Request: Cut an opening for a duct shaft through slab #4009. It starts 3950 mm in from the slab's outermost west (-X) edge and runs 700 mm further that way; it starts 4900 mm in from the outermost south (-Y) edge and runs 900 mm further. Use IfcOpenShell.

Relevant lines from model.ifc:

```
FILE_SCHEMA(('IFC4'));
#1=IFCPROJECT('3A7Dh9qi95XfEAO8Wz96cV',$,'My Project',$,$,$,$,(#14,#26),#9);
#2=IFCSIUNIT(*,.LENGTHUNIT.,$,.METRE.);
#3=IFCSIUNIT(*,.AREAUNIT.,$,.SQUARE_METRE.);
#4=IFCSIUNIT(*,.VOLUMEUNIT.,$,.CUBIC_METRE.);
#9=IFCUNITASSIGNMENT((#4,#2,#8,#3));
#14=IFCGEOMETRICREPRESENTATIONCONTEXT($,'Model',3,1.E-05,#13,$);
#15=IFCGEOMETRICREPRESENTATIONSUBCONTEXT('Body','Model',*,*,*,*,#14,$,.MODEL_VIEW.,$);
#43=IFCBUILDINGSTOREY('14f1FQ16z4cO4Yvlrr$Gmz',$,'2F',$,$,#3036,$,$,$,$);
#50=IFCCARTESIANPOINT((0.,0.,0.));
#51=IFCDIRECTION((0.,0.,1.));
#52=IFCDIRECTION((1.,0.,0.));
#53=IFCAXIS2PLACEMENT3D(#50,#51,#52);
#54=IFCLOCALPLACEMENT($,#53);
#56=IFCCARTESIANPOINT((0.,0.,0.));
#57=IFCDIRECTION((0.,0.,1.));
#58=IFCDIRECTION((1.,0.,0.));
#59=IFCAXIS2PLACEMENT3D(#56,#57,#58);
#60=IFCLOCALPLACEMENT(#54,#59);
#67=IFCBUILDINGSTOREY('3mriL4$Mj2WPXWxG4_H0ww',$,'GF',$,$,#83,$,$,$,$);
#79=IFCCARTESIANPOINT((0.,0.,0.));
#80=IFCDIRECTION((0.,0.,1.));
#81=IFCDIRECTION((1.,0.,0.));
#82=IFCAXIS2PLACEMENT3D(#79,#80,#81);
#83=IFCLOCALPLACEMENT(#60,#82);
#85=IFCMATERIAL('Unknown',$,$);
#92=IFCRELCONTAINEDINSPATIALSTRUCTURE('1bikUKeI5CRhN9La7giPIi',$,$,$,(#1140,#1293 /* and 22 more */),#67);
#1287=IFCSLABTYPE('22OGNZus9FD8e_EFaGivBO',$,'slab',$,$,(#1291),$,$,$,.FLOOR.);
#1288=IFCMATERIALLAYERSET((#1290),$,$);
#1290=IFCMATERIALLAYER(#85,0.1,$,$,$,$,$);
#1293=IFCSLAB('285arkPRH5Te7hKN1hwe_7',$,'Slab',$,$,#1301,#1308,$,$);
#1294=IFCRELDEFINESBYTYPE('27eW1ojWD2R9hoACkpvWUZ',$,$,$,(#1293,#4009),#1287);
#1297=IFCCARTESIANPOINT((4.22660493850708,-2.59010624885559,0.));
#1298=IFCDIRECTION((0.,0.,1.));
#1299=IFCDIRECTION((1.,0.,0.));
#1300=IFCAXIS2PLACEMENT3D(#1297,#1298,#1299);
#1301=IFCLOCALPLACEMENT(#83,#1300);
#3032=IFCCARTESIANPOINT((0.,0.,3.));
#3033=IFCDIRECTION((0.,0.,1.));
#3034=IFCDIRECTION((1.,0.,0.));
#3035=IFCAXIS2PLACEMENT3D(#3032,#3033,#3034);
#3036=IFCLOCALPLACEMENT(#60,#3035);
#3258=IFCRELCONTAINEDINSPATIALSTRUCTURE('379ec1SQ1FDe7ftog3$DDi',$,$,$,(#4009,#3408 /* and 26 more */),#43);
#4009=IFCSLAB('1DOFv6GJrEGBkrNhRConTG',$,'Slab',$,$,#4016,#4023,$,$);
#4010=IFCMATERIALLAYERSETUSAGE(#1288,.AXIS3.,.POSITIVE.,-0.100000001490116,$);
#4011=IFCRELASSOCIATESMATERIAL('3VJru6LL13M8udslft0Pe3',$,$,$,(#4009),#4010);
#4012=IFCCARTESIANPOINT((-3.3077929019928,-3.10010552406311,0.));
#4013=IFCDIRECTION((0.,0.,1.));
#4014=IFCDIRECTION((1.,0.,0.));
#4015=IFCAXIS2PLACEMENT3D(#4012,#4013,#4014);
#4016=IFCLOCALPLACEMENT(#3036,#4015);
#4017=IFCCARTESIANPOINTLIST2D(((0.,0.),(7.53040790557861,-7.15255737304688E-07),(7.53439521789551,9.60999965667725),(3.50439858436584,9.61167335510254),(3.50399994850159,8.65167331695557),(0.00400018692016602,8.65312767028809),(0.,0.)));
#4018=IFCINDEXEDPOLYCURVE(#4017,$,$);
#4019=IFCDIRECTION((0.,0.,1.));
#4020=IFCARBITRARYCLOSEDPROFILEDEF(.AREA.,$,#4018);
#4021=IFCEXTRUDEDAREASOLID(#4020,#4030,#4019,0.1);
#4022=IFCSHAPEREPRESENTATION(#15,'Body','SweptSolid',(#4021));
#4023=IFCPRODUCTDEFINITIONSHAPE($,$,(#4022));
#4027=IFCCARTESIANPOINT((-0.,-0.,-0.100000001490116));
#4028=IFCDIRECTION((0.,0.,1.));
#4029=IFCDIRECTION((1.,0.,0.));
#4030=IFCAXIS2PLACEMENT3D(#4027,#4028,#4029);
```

```python
import numpy as np
import ifcopenshell
import ifcopenshell.api.feature
import ifcopenshell.api.geometry
import ifcopenshell.api.root
import ifcopenshell.geom
import ifcopenshell.util.placement
import ifcopenshell.util.representation
import ifcopenshell.util.shape
import ifcopenshell.util.unit

model = ifcopenshell.open("model.ifc")
unit_scale = ifcopenshell.util.unit.calculate_unit_scale(model)
settings = ifcopenshell.geom.settings()


def volume(element):
    """Net volume in cubic metres, openings subtracted."""
    shape = ifcopenshell.geom.create_shape(settings, element)
    return ifcopenshell.util.shape.get_volume(shape.geometry)


slab = model.by_id(4009)
before = volume(slab)

# Extent in the slab's own axes, in metres. The edges named are its -X and -Y sides.
slab_shape = ifcopenshell.geom.create_shape(settings, slab)
vertices = ifcopenshell.util.shape.get_vertices(slab_shape.geometry)
x_min, y_min, bottom = vertices.min(axis=0)
top = vertices[:, 2].max()

opening = ifcopenshell.api.root.create_entity(model, ifc_class="IfcOpeningElement", name="Duct shaft opening", predefined_type="OPENING")
context = ifcopenshell.util.representation.get_context(model, "Model", "Body", "MODEL_VIEW")
width, depth = 0.7, 0.9
outline = [(0.0, 0.0), (width, 0.0), (width, depth), (0.0, depth), (0.0, 0.0)]
# Overshoot both faces by 50 mm so the cut is clean.
shape = ifcopenshell.api.geometry.add_slab_representation(
    model, context=context, depth=top - bottom + 0.1, polyline=outline
)
ifcopenshell.api.geometry.assign_representation(model, product=opening, representation=shape)

matrix = ifcopenshell.util.placement.get_local_placement(slab.ObjectPlacement)
matrix[:, 3] = matrix @ np.append(np.array([x_min + 3.95, y_min + 4.9, bottom - 0.05]) / unit_scale, 1.0)
ifcopenshell.api.geometry.edit_object_placement(model, product=opening, matrix=matrix, is_si=False)
ifcopenshell.api.feature.add_feature(model, feature=opening, element=slab)

after = volume(slab)

print(f"slab volume {before:.3f} -> {after:.3f} m3")

model.write("model_edited.ifc")
```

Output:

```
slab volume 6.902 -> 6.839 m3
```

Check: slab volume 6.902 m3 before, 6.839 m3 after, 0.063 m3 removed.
